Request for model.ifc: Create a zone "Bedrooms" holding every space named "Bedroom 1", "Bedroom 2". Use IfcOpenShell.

First a look at what the model holds.

```python
import ifcopenshell

model = ifcopenshell.open("model.ifc")
print(model.schema)
seen = {}
for space in model.by_type("IfcSpace"):
    seen[space.LongName] = seen.get(space.LongName, 0) + 1
for name, count in sorted(seen.items(), key=str):
    print(count, "x", name)
print("zones:", [z.Name for z in model.by_type("IfcZone")][:20])
```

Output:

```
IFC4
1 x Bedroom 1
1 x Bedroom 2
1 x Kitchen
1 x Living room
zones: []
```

```python
import ifcopenshell
import ifcopenshell.api.group
import ifcopenshell.api.root

model = ifcopenshell.open("model.ifc")

names = {"Bedroom 1", "Bedroom 2"}
spaces = [s for s in model.by_type("IfcSpace") if s.LongName in names]

zone = ifcopenshell.api.root.create_entity(model, ifc_class="IfcZone", name="Bedrooms")
ifcopenshell.api.group.assign_group(model, products=spaces, group=zone)
print(len(spaces), "spaces in", zone.Name)

model.write("model_rev.ifc")
```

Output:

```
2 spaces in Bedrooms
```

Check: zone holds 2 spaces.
